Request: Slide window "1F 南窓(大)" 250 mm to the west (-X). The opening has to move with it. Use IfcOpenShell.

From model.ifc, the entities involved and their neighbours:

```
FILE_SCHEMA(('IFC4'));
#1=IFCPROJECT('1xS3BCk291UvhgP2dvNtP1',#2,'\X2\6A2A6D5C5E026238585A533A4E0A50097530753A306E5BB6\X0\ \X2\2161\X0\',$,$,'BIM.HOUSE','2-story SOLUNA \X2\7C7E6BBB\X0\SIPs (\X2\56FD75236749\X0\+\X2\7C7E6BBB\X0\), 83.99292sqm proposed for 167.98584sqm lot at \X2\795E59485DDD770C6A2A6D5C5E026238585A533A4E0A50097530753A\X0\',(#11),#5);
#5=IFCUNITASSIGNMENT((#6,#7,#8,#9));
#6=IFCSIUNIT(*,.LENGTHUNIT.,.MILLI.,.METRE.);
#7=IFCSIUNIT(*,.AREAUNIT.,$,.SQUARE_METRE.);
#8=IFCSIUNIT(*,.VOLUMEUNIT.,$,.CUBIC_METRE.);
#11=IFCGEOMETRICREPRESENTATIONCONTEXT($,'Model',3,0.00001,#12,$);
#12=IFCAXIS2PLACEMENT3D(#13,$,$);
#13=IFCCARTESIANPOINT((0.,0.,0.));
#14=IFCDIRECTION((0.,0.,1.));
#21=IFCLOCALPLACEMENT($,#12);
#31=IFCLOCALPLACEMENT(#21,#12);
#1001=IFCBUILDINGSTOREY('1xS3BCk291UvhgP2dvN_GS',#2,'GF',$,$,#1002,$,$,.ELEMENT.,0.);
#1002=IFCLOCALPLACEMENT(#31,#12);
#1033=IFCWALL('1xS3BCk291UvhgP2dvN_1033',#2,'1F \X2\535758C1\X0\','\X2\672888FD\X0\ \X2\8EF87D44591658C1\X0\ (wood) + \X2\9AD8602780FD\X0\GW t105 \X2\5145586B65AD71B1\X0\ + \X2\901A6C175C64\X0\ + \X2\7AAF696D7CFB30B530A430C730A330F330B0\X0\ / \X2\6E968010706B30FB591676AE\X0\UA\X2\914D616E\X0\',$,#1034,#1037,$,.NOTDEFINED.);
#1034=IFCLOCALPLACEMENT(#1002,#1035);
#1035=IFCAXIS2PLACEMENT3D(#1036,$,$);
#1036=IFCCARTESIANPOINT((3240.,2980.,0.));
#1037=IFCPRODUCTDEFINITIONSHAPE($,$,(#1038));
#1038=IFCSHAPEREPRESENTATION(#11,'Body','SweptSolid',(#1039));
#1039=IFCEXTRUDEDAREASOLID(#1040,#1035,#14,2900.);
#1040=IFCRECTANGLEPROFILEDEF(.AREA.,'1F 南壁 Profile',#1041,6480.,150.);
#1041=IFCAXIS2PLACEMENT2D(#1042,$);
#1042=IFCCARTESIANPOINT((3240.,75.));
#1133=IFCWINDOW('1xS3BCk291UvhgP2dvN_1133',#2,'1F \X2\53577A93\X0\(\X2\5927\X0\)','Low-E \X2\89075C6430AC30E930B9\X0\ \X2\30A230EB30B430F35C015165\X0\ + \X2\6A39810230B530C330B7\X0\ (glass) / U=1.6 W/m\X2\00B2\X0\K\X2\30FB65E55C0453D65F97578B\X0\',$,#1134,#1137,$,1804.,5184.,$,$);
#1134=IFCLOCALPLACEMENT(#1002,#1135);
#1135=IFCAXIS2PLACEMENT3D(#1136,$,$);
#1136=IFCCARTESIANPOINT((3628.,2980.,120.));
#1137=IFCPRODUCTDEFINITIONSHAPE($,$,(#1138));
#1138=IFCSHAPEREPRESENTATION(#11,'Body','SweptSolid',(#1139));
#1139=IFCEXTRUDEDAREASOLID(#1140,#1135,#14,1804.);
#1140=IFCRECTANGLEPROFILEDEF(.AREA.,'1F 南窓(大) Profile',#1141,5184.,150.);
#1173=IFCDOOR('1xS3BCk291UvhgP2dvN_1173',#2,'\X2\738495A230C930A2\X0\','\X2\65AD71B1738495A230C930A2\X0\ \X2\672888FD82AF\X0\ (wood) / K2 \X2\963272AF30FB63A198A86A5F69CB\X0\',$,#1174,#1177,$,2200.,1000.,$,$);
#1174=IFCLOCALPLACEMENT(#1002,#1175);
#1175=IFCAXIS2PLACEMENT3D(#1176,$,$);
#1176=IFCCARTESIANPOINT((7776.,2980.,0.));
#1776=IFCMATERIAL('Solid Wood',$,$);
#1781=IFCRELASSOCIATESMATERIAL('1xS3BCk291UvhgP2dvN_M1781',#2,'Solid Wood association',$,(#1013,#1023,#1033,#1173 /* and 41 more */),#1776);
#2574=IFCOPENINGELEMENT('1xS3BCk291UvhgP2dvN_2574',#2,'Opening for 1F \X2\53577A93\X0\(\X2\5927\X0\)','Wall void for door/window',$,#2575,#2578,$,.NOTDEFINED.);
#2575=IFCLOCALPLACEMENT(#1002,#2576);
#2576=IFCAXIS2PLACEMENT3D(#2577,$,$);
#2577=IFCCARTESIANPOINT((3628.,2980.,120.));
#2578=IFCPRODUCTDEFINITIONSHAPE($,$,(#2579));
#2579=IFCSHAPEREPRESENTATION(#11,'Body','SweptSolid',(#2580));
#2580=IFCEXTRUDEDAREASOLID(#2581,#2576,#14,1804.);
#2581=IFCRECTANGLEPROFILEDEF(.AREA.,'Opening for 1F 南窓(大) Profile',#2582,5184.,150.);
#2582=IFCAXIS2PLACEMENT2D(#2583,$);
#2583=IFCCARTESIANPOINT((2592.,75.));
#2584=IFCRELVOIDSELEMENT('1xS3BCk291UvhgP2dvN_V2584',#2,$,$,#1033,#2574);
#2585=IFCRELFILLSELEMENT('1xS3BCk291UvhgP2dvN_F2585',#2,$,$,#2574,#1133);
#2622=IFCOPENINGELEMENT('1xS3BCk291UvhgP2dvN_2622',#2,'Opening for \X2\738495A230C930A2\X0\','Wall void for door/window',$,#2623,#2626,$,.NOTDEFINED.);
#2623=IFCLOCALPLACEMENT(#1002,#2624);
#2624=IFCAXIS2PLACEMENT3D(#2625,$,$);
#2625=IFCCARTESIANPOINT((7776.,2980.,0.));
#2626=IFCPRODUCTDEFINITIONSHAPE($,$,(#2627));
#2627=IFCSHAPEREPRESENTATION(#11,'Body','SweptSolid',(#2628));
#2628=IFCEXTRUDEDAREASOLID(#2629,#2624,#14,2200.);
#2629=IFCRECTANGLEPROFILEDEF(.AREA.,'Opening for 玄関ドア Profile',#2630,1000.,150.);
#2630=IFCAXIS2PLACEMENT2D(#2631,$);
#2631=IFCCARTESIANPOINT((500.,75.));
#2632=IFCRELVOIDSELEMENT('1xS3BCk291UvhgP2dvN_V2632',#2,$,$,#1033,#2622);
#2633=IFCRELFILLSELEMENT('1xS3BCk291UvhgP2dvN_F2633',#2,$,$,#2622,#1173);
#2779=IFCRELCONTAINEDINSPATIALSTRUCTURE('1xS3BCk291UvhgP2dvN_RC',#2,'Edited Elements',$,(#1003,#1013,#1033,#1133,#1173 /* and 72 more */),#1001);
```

```python
import ifcopenshell
import ifcopenshell.api.geometry
import ifcopenshell.util.placement
import ifcopenshell.util.unit

model = ifcopenshell.open("model.ifc")
unit_scale = ifcopenshell.util.unit.calculate_unit_scale(model)

window = model.by_guid("1xS3BCk291UvhgP2dvN_1133")
opening = window.FillsVoids[0].RelatingOpeningElement
wall = opening.VoidsElements[0].RelatingBuildingElement

wall_matrix = ifcopenshell.util.placement.get_local_placement(wall.ObjectPlacement)
shift = wall_matrix[:3, 0] * -0.25 / unit_scale
before = ifcopenshell.util.placement.get_local_placement(window.ObjectPlacement)[:3, 3].copy()

# The window is not placed relative to its opening, so move both.
for product in (opening, window):
    matrix = ifcopenshell.util.placement.get_local_placement(product.ObjectPlacement)
    matrix[:3, 3] += shift
    ifcopenshell.api.geometry.edit_object_placement(model, product=product, matrix=matrix, is_si=False)

after = ifcopenshell.util.placement.get_local_placement(window.ObjectPlacement)[:3, 3]
print("window moved by", (after - before).round(3) + 0.0)

model.write("model_edited.ifc")
```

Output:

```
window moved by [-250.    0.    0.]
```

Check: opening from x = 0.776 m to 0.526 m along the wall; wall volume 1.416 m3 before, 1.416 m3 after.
